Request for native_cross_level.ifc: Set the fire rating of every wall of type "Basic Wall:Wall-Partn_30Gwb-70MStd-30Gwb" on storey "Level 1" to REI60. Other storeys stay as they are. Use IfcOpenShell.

First a look at what the model holds.

```python
import ifcopenshell
import ifcopenshell.util.element

model = ifcopenshell.open("native_cross_level.ifc")
print(model.schema)
storey = next(s for s in model.by_type("IfcBuildingStorey") if s.Name == "Level 1")
walls = [e for e in ifcopenshell.util.element.get_decomposition(storey) if e.is_a("IfcWall")]
seen = {}
for e in walls:
    element_type = ifcopenshell.util.element.get_type(e)
    key = (element_type.Name if element_type != e and element_type else None, ifcopenshell.util.element.get_pset(e, "Pset_WallCommon", "FireRating"))
    seen[key] = seen.get(key, 0) + 1
for (name, value), count in sorted(seen.items(), key=str):
    print(count, "x", name, "|", value)
```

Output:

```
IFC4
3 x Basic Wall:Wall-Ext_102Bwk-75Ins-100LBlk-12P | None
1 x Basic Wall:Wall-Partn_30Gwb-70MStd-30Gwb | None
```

```python
import ifcopenshell
import ifcopenshell.api.pset
import ifcopenshell.util.element

model = ifcopenshell.open("native_cross_level.ifc")

storey = next(s for s in model.by_type("IfcBuildingStorey") if s.Name == "Level 1")
walls = [e for e in ifcopenshell.util.element.get_decomposition(storey) if e.is_a("IfcWall")]

count = 0
for e in walls:
    element_type = ifcopenshell.util.element.get_type(e)
    if element_type in (None, e) or element_type.Name != "Basic Wall:Wall-Partn_30Gwb-70MStd-30Gwb":
        continue
    # add_pset returns the element's existing set when there is one.
    pset = ifcopenshell.api.pset.add_pset(model, product=e, name="Pset_WallCommon")
    ifcopenshell.api.pset.edit_pset(model, pset=pset, properties={"FireRating": "REI60"})
    count += 1

print(count, "walls updated")

model.write("native_cross_level_rev.ifc")
```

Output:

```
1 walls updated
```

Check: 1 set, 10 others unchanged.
